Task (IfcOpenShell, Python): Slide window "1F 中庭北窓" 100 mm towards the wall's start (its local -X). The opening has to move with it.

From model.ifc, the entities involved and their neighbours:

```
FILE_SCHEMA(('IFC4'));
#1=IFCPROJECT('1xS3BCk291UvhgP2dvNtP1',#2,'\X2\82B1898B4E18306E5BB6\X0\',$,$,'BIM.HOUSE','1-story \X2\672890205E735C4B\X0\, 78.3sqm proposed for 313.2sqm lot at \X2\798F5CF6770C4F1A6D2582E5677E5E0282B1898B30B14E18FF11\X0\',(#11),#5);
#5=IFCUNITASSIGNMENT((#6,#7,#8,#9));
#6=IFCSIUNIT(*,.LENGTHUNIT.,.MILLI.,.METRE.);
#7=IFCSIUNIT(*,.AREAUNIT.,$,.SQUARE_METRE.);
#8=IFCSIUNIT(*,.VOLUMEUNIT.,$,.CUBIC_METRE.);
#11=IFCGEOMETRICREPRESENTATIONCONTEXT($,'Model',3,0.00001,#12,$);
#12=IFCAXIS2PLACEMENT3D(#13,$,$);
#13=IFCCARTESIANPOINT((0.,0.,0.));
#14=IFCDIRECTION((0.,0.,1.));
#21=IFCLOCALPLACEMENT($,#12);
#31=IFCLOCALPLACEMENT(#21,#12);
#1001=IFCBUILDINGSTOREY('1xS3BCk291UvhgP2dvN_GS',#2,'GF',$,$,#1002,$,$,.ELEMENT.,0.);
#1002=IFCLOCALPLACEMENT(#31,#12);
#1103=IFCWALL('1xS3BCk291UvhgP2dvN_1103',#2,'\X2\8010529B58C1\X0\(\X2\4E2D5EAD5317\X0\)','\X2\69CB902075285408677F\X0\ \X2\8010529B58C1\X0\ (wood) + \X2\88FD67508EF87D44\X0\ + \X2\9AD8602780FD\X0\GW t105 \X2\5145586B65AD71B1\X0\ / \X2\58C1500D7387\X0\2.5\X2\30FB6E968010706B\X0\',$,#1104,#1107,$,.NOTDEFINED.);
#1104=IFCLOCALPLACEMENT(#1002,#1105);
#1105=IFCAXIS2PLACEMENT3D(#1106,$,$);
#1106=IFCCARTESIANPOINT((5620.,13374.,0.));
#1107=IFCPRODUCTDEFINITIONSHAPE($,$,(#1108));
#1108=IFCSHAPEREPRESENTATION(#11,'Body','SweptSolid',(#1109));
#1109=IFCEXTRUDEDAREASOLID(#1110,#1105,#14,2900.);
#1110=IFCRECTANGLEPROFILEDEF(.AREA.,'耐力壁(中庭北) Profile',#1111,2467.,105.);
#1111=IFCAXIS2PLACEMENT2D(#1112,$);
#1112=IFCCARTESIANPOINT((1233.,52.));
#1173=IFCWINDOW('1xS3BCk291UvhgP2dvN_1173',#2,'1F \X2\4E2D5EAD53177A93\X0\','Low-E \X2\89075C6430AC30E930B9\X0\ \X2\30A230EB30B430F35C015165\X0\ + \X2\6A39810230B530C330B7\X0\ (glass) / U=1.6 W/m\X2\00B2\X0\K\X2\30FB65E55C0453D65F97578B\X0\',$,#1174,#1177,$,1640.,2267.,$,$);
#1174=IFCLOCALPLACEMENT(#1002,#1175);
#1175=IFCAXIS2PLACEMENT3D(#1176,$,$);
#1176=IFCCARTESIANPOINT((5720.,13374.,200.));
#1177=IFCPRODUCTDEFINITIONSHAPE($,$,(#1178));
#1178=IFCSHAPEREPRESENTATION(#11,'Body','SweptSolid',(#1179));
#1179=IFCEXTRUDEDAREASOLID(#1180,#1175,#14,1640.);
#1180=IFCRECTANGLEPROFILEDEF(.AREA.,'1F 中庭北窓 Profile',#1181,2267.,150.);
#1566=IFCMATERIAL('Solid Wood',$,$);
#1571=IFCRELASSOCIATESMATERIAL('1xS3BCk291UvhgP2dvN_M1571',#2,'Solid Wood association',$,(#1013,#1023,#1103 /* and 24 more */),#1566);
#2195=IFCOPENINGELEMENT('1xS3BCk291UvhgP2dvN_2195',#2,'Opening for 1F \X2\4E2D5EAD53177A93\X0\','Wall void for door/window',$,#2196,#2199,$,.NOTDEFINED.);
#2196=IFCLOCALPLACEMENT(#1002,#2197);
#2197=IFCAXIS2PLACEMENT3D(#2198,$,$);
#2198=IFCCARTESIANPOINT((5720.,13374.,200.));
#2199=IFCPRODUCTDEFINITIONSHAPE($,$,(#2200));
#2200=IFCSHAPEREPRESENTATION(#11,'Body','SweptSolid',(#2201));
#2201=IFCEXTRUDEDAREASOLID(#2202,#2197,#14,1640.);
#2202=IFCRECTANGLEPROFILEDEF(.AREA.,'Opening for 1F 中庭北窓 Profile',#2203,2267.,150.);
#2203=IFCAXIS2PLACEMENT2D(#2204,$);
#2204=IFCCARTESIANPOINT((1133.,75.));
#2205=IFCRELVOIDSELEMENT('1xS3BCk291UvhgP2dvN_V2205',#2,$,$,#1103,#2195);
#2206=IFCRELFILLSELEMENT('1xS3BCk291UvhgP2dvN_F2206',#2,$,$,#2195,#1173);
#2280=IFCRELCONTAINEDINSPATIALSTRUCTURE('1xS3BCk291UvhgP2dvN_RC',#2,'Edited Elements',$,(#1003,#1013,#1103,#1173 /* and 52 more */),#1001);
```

```python
import ifcopenshell
import ifcopenshell.api.geometry
import ifcopenshell.util.placement
import ifcopenshell.util.unit

model = ifcopenshell.open("model.ifc")
unit_scale = ifcopenshell.util.unit.calculate_unit_scale(model)

window = model.by_guid("1xS3BCk291UvhgP2dvN_1173")
opening = window.FillsVoids[0].RelatingOpeningElement
wall = opening.VoidsElements[0].RelatingBuildingElement

wall_matrix = ifcopenshell.util.placement.get_local_placement(wall.ObjectPlacement)
shift = wall_matrix[:3, 0] * -0.1 / unit_scale
before = ifcopenshell.util.placement.get_local_placement(window.ObjectPlacement)[:3, 3].copy()

# The window is not placed relative to its opening, so move both.
for product in (opening, window):
    matrix = ifcopenshell.util.placement.get_local_placement(product.ObjectPlacement)
    matrix[:3, 3] += shift
    ifcopenshell.api.geometry.edit_object_placement(model, product=product, matrix=matrix, is_si=False)

after = ifcopenshell.util.placement.get_local_placement(window.ObjectPlacement)[:3, 3]
print("window moved by", (after - before).round(3) + 0.0)

model.write("model_updated.ifc")
```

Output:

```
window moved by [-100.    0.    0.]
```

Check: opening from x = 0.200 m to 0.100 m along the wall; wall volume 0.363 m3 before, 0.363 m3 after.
